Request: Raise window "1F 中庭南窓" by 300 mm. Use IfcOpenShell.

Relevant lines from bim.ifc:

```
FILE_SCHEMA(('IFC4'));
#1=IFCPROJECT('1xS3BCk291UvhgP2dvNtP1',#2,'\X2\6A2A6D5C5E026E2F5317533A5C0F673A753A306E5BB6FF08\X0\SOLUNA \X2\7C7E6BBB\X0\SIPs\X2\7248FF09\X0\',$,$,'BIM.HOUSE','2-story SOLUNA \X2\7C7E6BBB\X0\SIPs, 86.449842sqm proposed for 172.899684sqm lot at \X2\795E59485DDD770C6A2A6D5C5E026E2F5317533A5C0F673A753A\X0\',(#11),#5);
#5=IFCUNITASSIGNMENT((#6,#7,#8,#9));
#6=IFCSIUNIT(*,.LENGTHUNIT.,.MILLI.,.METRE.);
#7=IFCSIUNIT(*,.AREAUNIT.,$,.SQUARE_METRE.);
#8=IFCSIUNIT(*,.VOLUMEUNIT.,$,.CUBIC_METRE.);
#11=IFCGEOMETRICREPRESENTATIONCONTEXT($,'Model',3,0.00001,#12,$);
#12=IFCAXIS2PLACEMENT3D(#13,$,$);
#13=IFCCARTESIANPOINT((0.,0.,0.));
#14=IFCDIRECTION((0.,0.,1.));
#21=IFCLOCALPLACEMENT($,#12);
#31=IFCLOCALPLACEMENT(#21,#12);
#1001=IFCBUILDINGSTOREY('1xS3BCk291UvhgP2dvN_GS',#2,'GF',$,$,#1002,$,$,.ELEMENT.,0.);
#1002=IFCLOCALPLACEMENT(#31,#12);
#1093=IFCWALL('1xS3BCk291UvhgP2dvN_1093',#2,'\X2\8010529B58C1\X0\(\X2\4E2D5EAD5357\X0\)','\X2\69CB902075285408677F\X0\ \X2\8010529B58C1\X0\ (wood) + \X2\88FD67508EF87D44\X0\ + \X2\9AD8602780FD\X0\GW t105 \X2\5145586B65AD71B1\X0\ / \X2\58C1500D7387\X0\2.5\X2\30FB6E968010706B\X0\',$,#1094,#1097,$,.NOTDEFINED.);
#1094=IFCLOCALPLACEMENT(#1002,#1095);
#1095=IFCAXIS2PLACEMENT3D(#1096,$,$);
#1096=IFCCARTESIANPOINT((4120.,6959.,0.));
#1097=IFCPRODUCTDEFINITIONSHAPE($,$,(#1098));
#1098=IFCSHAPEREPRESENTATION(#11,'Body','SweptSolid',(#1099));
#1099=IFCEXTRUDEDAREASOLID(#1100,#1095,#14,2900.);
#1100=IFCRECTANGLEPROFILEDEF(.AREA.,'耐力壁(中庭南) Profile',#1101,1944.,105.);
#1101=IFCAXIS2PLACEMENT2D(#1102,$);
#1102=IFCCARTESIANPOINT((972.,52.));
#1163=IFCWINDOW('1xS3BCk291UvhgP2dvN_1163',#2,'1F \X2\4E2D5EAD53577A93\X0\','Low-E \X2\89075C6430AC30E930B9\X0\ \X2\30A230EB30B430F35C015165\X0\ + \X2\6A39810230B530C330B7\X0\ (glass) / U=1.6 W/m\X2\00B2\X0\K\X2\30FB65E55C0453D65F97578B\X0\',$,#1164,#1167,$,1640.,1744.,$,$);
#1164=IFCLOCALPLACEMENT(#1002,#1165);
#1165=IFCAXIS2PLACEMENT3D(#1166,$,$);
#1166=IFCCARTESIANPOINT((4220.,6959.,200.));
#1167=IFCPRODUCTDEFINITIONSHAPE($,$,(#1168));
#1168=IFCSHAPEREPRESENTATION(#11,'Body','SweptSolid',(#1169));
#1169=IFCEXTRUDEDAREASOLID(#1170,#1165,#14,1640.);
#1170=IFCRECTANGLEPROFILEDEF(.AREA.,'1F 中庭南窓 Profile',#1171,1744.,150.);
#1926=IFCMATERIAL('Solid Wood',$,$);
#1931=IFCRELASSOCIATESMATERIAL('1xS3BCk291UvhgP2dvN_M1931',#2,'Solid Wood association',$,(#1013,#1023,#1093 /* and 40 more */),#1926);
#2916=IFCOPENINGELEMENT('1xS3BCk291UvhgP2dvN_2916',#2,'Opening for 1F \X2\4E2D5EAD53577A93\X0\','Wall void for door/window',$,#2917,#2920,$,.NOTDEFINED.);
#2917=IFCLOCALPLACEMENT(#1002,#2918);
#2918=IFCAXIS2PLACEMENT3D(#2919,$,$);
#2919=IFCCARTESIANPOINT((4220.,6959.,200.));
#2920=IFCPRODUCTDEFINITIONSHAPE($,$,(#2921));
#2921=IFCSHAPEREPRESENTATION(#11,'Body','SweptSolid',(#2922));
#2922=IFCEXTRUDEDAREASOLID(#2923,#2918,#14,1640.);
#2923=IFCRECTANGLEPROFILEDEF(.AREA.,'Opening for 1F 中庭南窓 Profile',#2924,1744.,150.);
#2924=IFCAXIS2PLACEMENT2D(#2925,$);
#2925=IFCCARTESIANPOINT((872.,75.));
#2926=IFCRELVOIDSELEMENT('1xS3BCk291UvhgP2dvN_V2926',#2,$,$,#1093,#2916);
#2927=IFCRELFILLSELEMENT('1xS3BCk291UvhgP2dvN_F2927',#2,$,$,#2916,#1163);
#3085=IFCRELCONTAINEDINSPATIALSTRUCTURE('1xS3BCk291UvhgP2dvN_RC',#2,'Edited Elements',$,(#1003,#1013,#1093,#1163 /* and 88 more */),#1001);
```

```python
import numpy as np
import ifcopenshell
import ifcopenshell.api.geometry
import ifcopenshell.util.placement
import ifcopenshell.util.unit

model = ifcopenshell.open("bim.ifc")
unit_scale = ifcopenshell.util.unit.calculate_unit_scale(model)

window = model.by_guid("1xS3BCk291UvhgP2dvN_1163")
opening = window.FillsVoids[0].RelatingOpeningElement
dz = 300.0

shift = np.array([0.0, 0.0, dz])
# The window is not placed relative to its opening, so move both.
for product in (opening, window):
    matrix = ifcopenshell.util.placement.get_local_placement(product.ObjectPlacement)
    matrix[:3, 3] += shift
    ifcopenshell.api.geometry.edit_object_placement(model, product=product, matrix=matrix, is_si=False)

print(f"moved by {dz * unit_scale:+.3f} m")

model.write("bim_v2.ifc")
```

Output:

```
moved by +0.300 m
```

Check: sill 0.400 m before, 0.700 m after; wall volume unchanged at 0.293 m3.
